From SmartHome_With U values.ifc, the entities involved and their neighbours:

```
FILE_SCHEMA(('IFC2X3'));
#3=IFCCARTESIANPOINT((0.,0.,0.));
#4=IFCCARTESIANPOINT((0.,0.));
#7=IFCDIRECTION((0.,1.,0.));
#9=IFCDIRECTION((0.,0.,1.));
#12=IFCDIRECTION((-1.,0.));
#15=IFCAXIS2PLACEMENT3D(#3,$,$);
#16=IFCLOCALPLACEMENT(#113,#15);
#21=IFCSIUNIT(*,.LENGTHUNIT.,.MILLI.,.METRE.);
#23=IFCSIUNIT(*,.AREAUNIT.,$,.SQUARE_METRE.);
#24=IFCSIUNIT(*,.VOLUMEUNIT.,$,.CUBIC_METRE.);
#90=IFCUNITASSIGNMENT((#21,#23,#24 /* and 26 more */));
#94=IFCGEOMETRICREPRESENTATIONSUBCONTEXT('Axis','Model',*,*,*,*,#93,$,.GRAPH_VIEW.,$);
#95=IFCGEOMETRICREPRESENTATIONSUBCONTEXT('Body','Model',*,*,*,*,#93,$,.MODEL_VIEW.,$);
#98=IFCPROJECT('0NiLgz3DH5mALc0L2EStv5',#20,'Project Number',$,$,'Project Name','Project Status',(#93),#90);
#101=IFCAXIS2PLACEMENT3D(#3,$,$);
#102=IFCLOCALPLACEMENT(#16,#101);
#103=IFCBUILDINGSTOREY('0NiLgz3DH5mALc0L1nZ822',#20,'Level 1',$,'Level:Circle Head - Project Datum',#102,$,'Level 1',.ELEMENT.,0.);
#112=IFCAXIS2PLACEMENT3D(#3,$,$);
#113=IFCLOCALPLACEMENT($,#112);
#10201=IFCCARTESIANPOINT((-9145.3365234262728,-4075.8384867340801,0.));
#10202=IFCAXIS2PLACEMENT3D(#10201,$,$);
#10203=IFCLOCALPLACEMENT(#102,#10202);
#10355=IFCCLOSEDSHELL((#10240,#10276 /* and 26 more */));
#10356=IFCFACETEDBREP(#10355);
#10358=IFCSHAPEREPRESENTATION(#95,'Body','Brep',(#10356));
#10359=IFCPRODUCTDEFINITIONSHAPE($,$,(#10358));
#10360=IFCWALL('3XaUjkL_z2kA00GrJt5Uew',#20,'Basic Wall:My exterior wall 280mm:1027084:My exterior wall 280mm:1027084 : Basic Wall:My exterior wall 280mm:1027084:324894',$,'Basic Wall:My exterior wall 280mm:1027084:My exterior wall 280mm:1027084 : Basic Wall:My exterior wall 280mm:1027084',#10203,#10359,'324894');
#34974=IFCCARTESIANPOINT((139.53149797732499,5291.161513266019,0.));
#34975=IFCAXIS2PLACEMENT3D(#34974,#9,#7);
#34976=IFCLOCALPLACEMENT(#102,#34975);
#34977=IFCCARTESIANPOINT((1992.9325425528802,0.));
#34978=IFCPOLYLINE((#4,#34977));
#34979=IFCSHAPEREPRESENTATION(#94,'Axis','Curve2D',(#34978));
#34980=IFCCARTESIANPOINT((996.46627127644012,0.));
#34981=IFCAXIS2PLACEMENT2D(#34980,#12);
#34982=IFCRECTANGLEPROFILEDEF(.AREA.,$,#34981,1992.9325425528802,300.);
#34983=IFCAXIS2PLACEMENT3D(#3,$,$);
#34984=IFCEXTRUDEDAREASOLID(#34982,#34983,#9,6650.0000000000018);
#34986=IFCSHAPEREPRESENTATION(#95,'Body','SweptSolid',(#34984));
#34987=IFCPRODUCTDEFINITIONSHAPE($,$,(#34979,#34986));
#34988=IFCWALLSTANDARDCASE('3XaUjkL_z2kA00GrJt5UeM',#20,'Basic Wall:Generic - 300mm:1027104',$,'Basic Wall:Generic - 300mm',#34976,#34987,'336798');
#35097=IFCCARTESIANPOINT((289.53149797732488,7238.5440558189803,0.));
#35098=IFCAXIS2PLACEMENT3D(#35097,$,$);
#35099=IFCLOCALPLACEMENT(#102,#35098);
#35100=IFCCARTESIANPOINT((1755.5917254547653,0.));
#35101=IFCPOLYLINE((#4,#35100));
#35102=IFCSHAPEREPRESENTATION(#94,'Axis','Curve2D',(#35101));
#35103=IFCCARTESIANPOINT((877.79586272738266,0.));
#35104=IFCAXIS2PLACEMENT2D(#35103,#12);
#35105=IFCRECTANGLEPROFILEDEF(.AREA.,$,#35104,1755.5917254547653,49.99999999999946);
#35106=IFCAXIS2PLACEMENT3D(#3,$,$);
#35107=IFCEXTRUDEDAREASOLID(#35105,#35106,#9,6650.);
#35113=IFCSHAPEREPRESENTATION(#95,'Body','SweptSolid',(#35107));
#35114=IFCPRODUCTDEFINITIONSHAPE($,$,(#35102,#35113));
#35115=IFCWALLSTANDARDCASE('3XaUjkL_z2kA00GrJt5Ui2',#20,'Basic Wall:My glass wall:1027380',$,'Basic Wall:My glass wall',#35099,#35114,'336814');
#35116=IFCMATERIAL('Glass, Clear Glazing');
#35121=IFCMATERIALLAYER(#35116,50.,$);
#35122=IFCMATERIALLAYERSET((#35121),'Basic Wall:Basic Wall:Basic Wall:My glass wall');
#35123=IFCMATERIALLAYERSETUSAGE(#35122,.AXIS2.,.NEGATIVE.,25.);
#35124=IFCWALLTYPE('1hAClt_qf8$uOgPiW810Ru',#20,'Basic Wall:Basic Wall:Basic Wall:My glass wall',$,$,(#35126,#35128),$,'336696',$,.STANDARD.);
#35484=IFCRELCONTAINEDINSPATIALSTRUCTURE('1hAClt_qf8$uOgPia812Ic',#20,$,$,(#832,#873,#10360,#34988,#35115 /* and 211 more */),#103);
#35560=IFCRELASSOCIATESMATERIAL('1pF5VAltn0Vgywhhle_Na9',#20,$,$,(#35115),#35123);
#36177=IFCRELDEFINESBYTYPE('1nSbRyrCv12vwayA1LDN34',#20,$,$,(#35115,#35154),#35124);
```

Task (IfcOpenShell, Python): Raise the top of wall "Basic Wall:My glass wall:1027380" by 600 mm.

```python
import ifcopenshell
import ifcopenshell.geom
import ifcopenshell.util.representation
import ifcopenshell.util.shape
import ifcopenshell.util.unit

model = ifcopenshell.open("SmartHome_With U values.ifc")
unit_scale = ifcopenshell.util.unit.calculate_unit_scale(model)
settings = ifcopenshell.geom.settings()


def volume(element):
    """Net volume in cubic metres, openings subtracted."""
    shape = ifcopenshell.geom.create_shape(settings, element)
    return ifcopenshell.util.shape.get_volume(shape.geometry)


wall = model.by_id(35115)
before = volume(wall)

body = ifcopenshell.util.representation.get_representation(wall, "Model", "Body")
solid = body.Items[0]
old_height = solid.Depth
solid.Depth += 0.6 / unit_scale
after = volume(wall)

print(f"height {old_height:g} -> {solid.Depth:g}, volume {before:.3f} -> {after:.3f} m3")

model.write("SmartHome_With U values_v2.ifc")
```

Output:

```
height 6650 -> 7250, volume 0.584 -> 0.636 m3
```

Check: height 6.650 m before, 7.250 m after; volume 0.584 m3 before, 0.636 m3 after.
